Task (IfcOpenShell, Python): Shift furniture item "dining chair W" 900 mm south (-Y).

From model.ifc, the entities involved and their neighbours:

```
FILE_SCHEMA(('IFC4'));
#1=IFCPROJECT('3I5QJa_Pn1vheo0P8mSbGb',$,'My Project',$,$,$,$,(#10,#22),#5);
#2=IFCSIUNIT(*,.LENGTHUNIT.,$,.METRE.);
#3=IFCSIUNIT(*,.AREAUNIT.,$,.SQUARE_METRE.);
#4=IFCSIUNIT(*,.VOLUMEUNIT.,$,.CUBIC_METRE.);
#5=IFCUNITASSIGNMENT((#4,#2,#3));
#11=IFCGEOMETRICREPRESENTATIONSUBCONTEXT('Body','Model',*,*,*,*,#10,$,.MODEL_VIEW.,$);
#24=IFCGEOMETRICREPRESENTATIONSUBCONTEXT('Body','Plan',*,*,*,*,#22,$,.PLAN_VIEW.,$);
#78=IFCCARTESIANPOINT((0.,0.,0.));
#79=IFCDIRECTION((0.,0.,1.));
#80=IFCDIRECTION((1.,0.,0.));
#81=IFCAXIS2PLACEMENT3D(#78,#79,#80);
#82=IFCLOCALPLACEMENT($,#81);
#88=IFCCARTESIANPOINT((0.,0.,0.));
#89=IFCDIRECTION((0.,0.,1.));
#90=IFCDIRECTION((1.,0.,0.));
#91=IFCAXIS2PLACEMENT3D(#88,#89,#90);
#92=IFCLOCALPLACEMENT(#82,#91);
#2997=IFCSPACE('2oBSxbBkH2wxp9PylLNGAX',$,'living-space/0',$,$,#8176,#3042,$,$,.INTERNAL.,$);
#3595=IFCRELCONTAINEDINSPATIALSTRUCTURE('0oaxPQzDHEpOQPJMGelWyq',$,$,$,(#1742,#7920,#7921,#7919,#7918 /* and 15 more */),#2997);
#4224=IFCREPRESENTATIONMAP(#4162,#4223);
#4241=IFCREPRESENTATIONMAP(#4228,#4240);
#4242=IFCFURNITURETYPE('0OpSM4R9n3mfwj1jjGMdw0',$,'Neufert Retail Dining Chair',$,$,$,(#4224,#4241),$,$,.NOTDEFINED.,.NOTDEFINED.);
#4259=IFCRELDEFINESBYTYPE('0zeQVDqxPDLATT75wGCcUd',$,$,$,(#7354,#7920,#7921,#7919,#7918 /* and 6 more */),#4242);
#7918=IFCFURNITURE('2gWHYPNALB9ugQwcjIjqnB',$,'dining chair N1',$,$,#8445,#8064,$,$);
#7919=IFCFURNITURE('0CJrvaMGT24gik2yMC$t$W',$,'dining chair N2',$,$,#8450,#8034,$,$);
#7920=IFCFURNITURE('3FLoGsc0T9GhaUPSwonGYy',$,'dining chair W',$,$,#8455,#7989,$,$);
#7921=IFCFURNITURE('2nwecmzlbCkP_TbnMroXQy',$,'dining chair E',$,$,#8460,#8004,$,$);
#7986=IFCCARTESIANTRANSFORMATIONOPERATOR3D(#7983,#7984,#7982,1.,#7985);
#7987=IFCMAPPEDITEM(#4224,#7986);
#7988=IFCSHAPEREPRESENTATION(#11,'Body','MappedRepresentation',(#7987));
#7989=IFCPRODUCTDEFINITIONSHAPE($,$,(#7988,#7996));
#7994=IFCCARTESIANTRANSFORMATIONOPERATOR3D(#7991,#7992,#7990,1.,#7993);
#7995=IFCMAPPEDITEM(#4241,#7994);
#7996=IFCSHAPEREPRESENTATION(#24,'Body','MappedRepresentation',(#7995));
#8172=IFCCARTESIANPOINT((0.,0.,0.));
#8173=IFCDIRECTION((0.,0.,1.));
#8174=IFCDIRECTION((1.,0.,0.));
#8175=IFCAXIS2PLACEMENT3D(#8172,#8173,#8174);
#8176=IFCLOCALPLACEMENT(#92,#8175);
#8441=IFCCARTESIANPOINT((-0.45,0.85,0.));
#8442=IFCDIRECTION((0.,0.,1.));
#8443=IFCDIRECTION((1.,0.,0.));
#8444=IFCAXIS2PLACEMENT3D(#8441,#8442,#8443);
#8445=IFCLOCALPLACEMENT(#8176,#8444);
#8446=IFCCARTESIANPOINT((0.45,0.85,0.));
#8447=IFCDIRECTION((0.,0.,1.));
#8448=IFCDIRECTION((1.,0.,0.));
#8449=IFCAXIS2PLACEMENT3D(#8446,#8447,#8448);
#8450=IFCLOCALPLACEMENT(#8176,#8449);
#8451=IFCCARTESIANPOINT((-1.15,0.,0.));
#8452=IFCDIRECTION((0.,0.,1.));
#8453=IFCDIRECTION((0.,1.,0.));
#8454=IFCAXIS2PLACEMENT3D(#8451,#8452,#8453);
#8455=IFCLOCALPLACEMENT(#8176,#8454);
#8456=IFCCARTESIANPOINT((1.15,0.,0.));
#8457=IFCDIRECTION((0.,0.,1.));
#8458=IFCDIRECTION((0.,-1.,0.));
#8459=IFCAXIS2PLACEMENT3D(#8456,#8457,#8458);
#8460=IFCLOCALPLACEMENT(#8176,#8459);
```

```python
import ifcopenshell
import ifcopenshell.api.geometry
import ifcopenshell.util.placement

model = ifcopenshell.open("model.ifc")

item = model.by_guid("3FLoGsc0T9GhaUPSwonGYy")
matrix = ifcopenshell.util.placement.get_local_placement(item.ObjectPlacement)
matrix[1, 3] -= 0.9
ifcopenshell.api.geometry.edit_object_placement(model, product=item, matrix=matrix, is_si=False)

print(ifcopenshell.util.placement.get_local_placement(item.ObjectPlacement).round(3) + 0.0)

model.write("model_updated.ifc")
```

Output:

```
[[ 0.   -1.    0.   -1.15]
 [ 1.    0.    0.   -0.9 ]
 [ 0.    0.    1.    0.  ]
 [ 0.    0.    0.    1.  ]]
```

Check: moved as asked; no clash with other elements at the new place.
